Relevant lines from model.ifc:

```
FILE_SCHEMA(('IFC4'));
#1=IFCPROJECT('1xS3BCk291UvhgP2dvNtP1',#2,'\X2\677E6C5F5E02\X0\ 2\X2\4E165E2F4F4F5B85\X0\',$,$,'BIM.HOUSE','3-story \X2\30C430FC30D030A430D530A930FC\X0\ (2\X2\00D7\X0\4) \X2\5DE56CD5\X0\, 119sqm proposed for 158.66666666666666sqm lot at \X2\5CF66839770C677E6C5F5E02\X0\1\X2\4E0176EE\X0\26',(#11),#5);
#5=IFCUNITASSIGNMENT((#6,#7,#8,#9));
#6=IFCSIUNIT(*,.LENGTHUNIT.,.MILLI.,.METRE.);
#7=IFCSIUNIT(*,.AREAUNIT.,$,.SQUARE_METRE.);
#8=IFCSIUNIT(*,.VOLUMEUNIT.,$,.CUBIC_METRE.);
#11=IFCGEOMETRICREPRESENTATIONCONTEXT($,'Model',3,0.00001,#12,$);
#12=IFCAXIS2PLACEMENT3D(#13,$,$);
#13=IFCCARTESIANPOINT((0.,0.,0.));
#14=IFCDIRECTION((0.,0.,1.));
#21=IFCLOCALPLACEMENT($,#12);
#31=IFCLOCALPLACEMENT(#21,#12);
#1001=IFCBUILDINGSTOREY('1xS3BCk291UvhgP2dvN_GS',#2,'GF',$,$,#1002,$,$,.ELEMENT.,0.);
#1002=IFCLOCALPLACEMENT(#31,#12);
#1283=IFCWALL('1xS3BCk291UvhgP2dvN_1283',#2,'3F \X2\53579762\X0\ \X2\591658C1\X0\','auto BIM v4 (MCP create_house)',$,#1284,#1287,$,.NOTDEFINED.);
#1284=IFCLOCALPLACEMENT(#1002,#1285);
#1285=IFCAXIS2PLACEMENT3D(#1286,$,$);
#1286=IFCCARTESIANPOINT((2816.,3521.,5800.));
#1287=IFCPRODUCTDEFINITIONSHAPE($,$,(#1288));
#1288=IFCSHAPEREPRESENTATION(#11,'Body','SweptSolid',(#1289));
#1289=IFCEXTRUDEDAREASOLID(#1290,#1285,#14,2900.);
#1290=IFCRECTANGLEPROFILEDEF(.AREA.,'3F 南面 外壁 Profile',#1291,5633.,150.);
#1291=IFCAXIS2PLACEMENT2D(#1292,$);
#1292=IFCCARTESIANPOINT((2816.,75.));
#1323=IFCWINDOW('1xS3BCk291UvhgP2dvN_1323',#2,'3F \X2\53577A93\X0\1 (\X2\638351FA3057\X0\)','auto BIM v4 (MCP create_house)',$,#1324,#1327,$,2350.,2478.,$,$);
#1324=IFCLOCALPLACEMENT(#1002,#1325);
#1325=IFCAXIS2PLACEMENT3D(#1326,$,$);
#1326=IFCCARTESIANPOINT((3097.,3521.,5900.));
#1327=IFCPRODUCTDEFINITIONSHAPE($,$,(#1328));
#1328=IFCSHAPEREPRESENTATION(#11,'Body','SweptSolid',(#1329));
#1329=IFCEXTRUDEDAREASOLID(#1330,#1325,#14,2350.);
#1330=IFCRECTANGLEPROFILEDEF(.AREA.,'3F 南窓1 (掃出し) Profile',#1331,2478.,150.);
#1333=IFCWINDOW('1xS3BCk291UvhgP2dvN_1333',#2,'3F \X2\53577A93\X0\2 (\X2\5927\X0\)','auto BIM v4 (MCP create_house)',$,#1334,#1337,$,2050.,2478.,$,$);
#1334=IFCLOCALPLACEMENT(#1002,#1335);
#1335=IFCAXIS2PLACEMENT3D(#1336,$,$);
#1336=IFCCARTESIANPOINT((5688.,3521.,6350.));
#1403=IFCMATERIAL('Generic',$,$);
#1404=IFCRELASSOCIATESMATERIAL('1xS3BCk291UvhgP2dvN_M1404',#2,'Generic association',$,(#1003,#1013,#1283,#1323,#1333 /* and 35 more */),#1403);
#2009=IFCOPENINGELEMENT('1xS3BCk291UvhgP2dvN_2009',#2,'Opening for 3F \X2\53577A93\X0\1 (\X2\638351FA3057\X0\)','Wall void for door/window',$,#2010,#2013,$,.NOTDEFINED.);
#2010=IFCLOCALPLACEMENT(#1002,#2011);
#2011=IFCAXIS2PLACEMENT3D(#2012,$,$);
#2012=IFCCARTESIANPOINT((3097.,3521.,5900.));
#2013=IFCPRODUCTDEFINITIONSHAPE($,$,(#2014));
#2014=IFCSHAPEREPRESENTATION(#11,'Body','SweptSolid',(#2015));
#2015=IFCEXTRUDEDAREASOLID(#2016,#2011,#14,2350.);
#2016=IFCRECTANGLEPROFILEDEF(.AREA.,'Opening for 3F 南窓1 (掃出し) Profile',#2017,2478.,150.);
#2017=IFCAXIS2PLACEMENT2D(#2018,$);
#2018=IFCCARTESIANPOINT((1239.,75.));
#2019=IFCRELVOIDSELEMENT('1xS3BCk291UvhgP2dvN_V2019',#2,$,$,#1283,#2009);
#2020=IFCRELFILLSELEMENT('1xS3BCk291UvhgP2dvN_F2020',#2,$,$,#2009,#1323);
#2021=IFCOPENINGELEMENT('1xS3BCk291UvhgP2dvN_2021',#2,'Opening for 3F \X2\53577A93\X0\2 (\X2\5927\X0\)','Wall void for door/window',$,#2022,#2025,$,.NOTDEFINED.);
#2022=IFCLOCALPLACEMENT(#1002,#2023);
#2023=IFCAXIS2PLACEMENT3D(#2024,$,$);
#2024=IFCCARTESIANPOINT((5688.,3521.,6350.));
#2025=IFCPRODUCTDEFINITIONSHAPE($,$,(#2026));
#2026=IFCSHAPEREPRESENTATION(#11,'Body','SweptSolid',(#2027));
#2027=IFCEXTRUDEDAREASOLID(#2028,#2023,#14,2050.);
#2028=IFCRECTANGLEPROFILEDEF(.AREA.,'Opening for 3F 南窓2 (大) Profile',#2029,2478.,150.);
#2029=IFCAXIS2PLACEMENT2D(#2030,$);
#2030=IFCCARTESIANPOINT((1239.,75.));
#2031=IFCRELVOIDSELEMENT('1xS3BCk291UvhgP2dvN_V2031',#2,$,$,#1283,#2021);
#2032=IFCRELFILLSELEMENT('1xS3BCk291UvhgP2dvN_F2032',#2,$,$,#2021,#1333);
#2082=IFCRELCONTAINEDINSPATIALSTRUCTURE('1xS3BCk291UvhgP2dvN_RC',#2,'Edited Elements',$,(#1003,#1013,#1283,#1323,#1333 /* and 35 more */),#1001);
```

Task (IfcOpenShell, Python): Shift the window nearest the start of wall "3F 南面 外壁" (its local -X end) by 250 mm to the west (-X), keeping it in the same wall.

```python
import ifcopenshell
import ifcopenshell.api.geometry
import ifcopenshell.util.placement

model = ifcopenshell.open("model.ifc")

window = model.by_guid("1xS3BCk291UvhgP2dvN_1323")
opening = window.FillsVoids[0].RelatingOpeningElement
wall = opening.VoidsElements[0].RelatingBuildingElement

wall_matrix = ifcopenshell.util.placement.get_local_placement(wall.ObjectPlacement)
shift = wall_matrix[:3, 0] * -250.0
before = ifcopenshell.util.placement.get_local_placement(window.ObjectPlacement)[:3, 3].copy()

# The window is not placed relative to its opening, so move both.
for product in (opening, window):
    matrix = ifcopenshell.util.placement.get_local_placement(product.ObjectPlacement)
    matrix[:3, 3] += shift
    ifcopenshell.api.geometry.edit_object_placement(model, product=product, matrix=matrix, is_si=False)

after = ifcopenshell.util.placement.get_local_placement(window.ObjectPlacement)[:3, 3]
print("window moved by", (after - before).round(3) + 0.0)

model.write("model_updated.ifc")
```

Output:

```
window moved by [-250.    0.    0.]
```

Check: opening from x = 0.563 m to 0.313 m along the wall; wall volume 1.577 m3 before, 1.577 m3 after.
